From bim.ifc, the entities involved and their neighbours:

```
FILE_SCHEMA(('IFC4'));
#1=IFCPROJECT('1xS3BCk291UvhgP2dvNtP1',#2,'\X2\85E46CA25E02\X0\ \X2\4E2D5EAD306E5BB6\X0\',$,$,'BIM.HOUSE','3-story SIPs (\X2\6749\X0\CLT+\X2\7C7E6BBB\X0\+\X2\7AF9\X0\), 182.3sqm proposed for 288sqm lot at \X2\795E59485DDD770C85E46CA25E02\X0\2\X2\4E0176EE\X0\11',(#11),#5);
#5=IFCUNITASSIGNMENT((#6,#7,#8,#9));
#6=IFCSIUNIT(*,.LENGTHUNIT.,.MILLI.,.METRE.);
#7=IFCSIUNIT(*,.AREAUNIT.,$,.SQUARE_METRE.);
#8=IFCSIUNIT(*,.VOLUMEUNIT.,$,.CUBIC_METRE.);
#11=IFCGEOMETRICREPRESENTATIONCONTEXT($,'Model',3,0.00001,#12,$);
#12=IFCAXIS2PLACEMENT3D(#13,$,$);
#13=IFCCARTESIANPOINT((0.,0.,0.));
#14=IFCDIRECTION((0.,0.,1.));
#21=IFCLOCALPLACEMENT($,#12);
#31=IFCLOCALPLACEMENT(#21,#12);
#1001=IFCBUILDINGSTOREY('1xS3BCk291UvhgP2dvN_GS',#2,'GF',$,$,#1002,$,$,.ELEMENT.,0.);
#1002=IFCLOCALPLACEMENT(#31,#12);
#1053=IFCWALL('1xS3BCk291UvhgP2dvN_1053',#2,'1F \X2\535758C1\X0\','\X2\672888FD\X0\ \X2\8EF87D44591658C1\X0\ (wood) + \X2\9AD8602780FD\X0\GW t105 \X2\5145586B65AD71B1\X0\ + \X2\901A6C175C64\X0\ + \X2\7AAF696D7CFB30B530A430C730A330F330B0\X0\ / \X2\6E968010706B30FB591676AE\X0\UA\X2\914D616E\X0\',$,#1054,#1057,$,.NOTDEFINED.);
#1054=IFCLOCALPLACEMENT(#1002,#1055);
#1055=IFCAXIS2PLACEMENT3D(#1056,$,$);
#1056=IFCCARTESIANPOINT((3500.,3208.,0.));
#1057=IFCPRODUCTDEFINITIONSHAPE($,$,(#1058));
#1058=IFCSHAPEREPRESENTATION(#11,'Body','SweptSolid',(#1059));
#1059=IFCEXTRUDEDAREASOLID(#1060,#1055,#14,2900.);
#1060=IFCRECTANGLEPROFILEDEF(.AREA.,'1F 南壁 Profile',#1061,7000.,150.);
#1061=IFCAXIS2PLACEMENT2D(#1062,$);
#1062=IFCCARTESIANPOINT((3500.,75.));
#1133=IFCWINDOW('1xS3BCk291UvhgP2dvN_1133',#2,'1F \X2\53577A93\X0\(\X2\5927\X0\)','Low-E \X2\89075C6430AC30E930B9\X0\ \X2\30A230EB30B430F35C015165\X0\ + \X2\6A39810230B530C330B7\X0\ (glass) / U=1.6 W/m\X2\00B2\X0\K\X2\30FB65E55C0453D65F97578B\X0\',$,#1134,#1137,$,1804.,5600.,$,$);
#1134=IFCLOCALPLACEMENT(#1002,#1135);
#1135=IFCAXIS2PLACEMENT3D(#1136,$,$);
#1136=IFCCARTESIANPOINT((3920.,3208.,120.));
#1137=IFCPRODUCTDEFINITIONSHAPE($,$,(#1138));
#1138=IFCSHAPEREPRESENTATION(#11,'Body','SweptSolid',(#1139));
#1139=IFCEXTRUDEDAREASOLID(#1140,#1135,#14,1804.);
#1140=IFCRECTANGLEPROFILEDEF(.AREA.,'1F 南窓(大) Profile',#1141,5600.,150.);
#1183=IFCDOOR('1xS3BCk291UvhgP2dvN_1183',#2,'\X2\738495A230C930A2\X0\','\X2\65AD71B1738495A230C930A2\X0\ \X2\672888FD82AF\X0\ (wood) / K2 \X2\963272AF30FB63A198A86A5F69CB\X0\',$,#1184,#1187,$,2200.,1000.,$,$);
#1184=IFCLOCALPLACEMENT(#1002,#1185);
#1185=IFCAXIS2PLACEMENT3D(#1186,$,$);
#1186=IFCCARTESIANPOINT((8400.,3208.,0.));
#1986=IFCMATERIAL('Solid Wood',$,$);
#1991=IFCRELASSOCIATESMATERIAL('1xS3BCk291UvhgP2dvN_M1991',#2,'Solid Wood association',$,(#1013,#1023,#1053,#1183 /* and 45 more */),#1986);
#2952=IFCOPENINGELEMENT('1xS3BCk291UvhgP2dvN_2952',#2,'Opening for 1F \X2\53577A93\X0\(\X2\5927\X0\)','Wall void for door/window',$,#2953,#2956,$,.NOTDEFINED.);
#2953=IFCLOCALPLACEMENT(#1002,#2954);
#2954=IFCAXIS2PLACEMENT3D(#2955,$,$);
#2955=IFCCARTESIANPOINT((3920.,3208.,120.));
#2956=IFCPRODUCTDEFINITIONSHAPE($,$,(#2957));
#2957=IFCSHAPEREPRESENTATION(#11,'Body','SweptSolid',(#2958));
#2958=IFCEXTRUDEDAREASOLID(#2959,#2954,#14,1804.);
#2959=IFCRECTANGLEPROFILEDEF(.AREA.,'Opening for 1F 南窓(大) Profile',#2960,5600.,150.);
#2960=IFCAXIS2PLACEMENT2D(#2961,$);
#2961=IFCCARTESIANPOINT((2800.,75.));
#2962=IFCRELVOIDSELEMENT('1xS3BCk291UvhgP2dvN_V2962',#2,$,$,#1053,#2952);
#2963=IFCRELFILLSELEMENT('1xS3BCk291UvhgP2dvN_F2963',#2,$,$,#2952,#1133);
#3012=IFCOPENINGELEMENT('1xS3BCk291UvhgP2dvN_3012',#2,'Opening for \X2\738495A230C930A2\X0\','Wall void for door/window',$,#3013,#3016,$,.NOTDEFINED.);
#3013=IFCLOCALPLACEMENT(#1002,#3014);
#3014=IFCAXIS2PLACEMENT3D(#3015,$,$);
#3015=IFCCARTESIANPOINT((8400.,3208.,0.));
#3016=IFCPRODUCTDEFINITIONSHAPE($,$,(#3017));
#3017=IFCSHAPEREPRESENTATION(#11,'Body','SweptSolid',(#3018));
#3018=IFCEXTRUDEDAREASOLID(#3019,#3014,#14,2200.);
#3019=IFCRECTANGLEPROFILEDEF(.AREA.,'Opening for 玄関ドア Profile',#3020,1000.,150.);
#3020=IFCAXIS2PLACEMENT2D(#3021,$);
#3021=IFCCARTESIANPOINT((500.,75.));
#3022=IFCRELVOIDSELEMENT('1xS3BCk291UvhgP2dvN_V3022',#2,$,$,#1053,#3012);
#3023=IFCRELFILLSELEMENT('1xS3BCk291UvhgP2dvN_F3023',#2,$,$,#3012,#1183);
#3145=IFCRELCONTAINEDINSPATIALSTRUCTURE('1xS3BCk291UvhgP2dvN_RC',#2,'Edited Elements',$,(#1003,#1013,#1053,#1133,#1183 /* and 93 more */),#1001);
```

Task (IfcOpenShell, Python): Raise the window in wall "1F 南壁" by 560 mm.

```python
import numpy as np
import ifcopenshell
import ifcopenshell.api.geometry
import ifcopenshell.util.placement
import ifcopenshell.util.unit

model = ifcopenshell.open("bim.ifc")
unit_scale = ifcopenshell.util.unit.calculate_unit_scale(model)

window = model.by_id(1133)
opening = window.FillsVoids[0].RelatingOpeningElement
dz = 0.56 / unit_scale

shift = np.array([0.0, 0.0, dz])
# The window is not placed relative to its opening, so move both.
for product in (opening, window):
    matrix = ifcopenshell.util.placement.get_local_placement(product.ObjectPlacement)
    matrix[:3, 3] += shift
    ifcopenshell.api.geometry.edit_object_placement(model, product=product, matrix=matrix, is_si=False)

print(f"moved by {dz * unit_scale:+.3f} m")

model.write("bim_v2.ifc")
```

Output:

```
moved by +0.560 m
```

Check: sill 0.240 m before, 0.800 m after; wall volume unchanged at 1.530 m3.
